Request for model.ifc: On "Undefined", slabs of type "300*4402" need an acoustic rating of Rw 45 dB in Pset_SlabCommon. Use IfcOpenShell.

First a look at what the model holds.

```python
import ifcopenshell
import ifcopenshell.util.element

model = ifcopenshell.open("model.ifc")
print(model.schema)
storey = next(s for s in model.by_type("IfcBuildingStorey") if s.Name == "Undefined")
slabs = [e for e in ifcopenshell.util.element.get_decomposition(storey) if e.is_a("IfcSlab")]
seen = {}
for e in slabs:
    element_type = ifcopenshell.util.element.get_type(e)
    key = (element_type.Name if element_type != e and element_type else None, ifcopenshell.util.element.get_pset(e, "Pset_SlabCommon", "AcousticRating"))
    seen[key] = seen.get(key, 0) + 1
for (name, value), count in sorted(seen.items(), key=str):
    print(count, "x", name, "|", value)
```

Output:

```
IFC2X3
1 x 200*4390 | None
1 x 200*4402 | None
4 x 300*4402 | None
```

```python
import ifcopenshell
import ifcopenshell.api.pset
import ifcopenshell.util.element

model = ifcopenshell.open("model.ifc")

storey = next(s for s in model.by_type("IfcBuildingStorey") if s.Name == "Undefined")
slabs = [e for e in ifcopenshell.util.element.get_decomposition(storey) if e.is_a("IfcSlab")]

count = 0
for e in slabs:
    element_type = ifcopenshell.util.element.get_type(e)
    if element_type in (None, e) or element_type.Name != "300*4402":
        continue
    # add_pset returns the element's existing set when there is one.
    pset = ifcopenshell.api.pset.add_pset(model, product=e, name="Pset_SlabCommon")
    ifcopenshell.api.pset.edit_pset(model, pset=pset, properties={"AcousticRating": "Rw 45 dB"})
    count += 1

print(count, "slabs updated")

model.write("model_rev.ifc")
```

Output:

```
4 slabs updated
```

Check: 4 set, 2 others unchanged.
